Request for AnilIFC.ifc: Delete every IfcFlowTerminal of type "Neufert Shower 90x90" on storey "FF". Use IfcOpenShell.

First a look at what the model holds.

```python
import ifcopenshell
import ifcopenshell.util.element

model = ifcopenshell.open("AnilIFC.ifc")
print(model.schema)
storey = next(s for s in model.by_type("IfcBuildingStorey") if s.Name == "FF")
terminals = [e for e in ifcopenshell.util.element.get_decomposition(storey) if e.is_a("IfcFlowTerminal")]
seen = {}
for e in terminals:
    element_type = ifcopenshell.util.element.get_type(e)
    name = element_type.Name if element_type not in (None, e) else None
    seen[name] = seen.get(name, 0) + 1
for name, count in sorted(seen.items(), key=str):
    print(count, "x", name)
```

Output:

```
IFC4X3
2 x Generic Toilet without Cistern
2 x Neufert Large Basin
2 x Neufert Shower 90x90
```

```python
import ifcopenshell
import ifcopenshell.api.root
import ifcopenshell.util.element

model = ifcopenshell.open("AnilIFC.ifc")

storey = next(s for s in model.by_type("IfcBuildingStorey") if s.Name == "FF")
terminals = [e for e in ifcopenshell.util.element.get_decomposition(storey) if e.is_a("IfcFlowTerminal")]
targets = [e for e in terminals if (t := ifcopenshell.util.element.get_type(e)) not in (None, e) and t.Name == "Neufert Shower 90x90"]

for e in targets:
    ifcopenshell.api.root.remove_product(model, product=e)
print(len(targets), "removed")

model.write("AnilIFC_updated.ifc")
```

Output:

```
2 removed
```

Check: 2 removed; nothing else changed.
